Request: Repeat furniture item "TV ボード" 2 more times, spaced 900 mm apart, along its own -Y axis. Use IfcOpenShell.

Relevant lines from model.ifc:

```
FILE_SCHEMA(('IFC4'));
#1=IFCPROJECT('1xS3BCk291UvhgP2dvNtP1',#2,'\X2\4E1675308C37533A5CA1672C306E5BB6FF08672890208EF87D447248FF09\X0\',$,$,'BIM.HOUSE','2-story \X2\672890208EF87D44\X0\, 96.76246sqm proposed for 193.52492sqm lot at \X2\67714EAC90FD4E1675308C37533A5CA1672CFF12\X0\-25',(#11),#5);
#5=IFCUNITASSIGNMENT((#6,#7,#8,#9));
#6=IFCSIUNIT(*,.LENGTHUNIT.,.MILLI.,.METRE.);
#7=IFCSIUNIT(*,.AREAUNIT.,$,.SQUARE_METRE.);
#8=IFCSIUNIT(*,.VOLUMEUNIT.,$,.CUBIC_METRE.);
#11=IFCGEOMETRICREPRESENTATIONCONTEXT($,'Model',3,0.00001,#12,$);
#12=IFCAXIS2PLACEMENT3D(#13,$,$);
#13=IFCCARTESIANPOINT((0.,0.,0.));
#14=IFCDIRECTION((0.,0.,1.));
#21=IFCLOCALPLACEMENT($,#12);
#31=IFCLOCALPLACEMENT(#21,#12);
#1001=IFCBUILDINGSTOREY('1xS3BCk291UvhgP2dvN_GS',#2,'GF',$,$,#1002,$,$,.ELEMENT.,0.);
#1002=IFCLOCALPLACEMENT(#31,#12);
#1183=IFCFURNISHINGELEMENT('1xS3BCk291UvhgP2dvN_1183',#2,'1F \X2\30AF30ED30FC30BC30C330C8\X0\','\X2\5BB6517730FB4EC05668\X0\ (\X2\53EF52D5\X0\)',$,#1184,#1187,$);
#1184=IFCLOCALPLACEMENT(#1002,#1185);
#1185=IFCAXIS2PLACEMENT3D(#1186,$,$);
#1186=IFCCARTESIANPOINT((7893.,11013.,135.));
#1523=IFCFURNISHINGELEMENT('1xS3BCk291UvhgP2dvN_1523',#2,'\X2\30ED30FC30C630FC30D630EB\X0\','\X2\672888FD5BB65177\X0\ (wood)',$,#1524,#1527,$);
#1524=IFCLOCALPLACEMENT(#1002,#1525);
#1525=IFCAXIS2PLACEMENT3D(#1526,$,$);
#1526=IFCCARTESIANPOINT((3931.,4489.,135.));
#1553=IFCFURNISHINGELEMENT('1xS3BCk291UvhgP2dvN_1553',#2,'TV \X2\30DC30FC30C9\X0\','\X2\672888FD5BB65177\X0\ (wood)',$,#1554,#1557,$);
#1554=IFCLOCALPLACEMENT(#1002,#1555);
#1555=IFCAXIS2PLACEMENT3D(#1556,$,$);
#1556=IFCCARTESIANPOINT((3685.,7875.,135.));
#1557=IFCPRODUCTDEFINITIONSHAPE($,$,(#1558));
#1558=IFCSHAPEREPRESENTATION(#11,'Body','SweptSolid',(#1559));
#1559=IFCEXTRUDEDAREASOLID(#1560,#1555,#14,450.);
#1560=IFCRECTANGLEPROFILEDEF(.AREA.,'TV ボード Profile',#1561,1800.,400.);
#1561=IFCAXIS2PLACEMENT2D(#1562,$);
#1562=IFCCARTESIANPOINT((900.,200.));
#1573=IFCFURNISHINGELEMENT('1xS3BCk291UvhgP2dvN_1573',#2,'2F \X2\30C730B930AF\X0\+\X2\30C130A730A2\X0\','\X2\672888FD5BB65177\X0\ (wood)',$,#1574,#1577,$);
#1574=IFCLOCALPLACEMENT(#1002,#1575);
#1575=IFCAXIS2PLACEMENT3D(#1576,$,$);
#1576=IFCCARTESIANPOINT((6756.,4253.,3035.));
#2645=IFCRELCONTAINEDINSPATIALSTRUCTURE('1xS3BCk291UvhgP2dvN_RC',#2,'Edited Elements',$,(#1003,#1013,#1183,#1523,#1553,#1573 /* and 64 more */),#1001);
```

```python
import ifcopenshell
import ifcopenshell.api.geometry
import ifcopenshell.api.root
import ifcopenshell.util.element
import ifcopenshell.util.placement

model = ifcopenshell.open("model.ifc")


def reuse_history(source, copy):
    """copy_class also copies each property set's owner history, people and application; keep the originals."""
    for rel in copy.IsDefinedBy:
        if rel.is_a("IfcRelDefinesByProperties") and (history := rel.RelatingPropertyDefinition.OwnerHistory):
            rel.RelatingPropertyDefinition.OwnerHistory = source.OwnerHistory
            ifcopenshell.util.element.remove_deep2(model, history)


source = model.by_guid("1xS3BCk291UvhgP2dvN_1553")
base = ifcopenshell.util.placement.get_local_placement(source.ObjectPlacement)
step = -base[:3, 1] * 900.0

for i in range(1, 3):
    copy = ifcopenshell.api.root.copy_class(model, product=source)
    copy.Representation = ifcopenshell.util.element.copy_deep(
        model, source.Representation, exclude=["IfcGeometricRepresentationContext", "IfcRepresentationMap"]
    )
    reuse_history(source, copy)
    matrix = base.copy()
    matrix[:3, 3] += i * step
    print("added at", matrix[:3, 3].round(3) + 0.0)
    ifcopenshell.api.geometry.edit_object_placement(model, product=copy, matrix=matrix, is_si=False)

model.write("model_updated.ifc")
```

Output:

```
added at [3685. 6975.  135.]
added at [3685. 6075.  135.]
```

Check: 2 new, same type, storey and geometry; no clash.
